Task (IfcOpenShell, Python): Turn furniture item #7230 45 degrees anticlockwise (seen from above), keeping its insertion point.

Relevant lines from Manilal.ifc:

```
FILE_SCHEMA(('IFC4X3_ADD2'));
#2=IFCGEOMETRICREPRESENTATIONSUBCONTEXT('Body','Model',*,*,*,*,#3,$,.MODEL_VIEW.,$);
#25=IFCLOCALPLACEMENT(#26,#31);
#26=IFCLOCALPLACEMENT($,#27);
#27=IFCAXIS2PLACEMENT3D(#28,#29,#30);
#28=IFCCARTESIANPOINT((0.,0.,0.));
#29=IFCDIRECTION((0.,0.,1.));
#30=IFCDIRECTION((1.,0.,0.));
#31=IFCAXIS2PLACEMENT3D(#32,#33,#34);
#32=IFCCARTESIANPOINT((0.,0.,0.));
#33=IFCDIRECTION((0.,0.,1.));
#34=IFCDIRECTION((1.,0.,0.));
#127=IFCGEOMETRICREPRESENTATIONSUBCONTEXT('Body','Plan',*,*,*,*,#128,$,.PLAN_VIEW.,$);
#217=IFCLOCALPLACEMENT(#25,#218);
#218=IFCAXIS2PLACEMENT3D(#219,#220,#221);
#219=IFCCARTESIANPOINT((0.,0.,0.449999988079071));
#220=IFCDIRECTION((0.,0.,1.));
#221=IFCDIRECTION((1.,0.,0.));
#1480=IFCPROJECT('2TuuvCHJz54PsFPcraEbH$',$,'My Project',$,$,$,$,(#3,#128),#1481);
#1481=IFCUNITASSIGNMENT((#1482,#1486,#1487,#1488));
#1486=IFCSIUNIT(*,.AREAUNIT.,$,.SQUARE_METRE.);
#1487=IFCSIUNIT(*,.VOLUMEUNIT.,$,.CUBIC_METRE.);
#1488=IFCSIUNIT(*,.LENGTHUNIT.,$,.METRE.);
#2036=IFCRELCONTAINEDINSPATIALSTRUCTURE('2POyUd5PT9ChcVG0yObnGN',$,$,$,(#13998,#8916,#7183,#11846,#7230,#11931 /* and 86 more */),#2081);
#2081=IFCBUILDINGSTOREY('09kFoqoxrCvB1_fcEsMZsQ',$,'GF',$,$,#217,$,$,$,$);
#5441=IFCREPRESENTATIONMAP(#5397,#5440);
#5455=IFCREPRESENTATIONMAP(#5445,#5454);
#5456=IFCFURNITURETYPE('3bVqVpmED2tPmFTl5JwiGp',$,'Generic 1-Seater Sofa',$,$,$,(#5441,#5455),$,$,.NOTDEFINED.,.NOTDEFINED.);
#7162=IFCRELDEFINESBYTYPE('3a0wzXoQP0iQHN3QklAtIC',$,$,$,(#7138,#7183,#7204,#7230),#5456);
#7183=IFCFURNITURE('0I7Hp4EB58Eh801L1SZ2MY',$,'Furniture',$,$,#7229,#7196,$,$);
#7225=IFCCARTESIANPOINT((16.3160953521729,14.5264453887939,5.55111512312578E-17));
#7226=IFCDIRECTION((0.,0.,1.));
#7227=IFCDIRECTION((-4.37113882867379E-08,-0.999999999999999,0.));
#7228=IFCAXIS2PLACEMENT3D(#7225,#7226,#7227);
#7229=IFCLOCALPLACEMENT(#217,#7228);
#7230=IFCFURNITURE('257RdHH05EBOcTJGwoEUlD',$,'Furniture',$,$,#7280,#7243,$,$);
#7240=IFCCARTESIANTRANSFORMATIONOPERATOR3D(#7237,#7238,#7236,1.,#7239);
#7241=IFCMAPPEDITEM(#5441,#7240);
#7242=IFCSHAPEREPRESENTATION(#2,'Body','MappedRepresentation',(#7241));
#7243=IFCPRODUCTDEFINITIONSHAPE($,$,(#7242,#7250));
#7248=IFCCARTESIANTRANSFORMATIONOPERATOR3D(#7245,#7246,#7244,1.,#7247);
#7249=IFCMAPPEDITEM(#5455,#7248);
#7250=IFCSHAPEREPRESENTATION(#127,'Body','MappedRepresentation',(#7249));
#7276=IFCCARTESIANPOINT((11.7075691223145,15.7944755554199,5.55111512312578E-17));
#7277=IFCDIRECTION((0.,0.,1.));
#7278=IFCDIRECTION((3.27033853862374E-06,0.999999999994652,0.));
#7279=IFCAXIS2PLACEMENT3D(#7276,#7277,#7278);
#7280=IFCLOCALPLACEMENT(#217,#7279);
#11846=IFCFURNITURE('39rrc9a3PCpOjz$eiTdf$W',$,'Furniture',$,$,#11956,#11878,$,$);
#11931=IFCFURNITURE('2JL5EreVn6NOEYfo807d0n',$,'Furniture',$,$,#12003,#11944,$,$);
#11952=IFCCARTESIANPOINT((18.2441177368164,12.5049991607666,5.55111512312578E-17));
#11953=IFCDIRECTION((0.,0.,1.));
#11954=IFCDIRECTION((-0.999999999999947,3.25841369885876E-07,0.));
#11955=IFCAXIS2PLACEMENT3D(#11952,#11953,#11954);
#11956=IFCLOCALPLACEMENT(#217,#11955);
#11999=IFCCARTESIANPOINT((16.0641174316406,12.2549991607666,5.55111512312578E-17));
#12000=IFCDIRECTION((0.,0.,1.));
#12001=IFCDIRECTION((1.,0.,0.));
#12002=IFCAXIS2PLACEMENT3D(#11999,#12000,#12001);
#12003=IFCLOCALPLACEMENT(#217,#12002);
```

```python
import ifcopenshell
import ifcopenshell.api.geometry
import ifcopenshell.util.placement

model = ifcopenshell.open("Manilal.ifc")

item = model.by_guid("257RdHH05EBOcTJGwoEUlD")
matrix = ifcopenshell.util.placement.get_local_placement(item.ObjectPlacement)
matrix = matrix @ ifcopenshell.util.placement.rotation(45, "Z")
ifcopenshell.api.geometry.edit_object_placement(model, product=item, matrix=matrix, is_si=False)

print(ifcopenshell.util.placement.get_local_placement(item.ObjectPlacement).round(3) + 0.0)

model.write("Manilal-out.ifc")
```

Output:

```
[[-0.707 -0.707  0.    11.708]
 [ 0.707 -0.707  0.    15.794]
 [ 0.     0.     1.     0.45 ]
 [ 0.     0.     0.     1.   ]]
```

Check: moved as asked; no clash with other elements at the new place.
